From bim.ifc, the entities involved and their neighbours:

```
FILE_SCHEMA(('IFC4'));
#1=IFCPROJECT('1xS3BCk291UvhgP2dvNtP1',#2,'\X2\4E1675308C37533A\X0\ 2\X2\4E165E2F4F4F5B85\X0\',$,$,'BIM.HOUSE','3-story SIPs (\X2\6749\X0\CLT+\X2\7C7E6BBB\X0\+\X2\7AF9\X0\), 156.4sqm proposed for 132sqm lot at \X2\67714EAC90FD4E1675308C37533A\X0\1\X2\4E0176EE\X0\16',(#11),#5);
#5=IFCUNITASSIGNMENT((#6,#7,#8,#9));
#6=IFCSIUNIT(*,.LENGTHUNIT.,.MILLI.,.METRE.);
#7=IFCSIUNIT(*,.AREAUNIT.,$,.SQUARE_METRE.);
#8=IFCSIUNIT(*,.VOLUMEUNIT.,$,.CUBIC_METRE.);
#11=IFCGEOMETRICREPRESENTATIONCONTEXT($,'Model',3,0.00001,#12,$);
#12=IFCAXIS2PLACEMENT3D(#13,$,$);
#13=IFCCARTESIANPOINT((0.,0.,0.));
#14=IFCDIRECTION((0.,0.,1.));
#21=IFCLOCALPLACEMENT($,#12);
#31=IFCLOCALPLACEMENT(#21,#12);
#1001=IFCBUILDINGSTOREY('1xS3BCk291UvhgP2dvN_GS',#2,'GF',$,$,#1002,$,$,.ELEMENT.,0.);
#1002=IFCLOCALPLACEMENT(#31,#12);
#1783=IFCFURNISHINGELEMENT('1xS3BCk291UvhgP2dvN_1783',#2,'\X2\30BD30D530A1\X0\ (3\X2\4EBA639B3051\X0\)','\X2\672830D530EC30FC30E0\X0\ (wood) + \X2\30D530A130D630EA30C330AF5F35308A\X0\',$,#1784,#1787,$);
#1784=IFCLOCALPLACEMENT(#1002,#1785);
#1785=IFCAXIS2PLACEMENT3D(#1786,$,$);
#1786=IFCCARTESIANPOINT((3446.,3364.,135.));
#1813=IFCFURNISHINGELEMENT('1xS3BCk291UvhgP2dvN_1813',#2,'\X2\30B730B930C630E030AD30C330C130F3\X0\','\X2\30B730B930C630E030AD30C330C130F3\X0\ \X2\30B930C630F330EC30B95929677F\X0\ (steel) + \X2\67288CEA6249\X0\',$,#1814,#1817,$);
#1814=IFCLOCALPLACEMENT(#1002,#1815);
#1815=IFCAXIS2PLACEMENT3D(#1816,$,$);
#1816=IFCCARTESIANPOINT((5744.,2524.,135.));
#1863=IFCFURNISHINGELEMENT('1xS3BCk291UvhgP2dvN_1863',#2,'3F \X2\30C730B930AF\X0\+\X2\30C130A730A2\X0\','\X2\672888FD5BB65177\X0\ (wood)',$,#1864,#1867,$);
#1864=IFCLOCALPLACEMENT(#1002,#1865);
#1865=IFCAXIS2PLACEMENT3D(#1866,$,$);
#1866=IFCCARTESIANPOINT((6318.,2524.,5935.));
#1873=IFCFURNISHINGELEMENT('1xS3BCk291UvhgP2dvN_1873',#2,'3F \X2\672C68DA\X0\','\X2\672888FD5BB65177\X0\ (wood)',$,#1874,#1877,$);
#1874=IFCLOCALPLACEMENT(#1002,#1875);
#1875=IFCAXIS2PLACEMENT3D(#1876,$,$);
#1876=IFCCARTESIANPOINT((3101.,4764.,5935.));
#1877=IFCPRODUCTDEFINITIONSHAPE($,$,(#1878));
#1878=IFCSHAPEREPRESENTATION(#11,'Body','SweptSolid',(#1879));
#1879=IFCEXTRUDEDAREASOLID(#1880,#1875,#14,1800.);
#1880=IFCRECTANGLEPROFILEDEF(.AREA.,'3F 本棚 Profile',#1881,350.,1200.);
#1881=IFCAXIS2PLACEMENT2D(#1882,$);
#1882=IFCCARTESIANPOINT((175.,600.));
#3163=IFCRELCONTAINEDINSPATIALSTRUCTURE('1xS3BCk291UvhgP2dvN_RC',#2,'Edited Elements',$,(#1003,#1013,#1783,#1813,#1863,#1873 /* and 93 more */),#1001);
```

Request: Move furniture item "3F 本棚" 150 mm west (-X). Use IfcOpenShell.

```python
import ifcopenshell
import ifcopenshell.api.geometry
import ifcopenshell.util.placement

model = ifcopenshell.open("bim.ifc")

item = model.by_guid("1xS3BCk291UvhgP2dvN_1873")
matrix = ifcopenshell.util.placement.get_local_placement(item.ObjectPlacement)
matrix[0, 3] -= 150.0
ifcopenshell.api.geometry.edit_object_placement(model, product=item, matrix=matrix, is_si=False)

print(ifcopenshell.util.placement.get_local_placement(item.ObjectPlacement).round(3) + 0.0)

model.write("bim_edited.ifc")
```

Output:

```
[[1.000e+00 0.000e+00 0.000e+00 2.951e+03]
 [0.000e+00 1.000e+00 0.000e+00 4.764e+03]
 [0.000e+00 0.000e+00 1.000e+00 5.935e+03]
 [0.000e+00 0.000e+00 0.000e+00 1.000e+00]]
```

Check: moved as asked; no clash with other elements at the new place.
